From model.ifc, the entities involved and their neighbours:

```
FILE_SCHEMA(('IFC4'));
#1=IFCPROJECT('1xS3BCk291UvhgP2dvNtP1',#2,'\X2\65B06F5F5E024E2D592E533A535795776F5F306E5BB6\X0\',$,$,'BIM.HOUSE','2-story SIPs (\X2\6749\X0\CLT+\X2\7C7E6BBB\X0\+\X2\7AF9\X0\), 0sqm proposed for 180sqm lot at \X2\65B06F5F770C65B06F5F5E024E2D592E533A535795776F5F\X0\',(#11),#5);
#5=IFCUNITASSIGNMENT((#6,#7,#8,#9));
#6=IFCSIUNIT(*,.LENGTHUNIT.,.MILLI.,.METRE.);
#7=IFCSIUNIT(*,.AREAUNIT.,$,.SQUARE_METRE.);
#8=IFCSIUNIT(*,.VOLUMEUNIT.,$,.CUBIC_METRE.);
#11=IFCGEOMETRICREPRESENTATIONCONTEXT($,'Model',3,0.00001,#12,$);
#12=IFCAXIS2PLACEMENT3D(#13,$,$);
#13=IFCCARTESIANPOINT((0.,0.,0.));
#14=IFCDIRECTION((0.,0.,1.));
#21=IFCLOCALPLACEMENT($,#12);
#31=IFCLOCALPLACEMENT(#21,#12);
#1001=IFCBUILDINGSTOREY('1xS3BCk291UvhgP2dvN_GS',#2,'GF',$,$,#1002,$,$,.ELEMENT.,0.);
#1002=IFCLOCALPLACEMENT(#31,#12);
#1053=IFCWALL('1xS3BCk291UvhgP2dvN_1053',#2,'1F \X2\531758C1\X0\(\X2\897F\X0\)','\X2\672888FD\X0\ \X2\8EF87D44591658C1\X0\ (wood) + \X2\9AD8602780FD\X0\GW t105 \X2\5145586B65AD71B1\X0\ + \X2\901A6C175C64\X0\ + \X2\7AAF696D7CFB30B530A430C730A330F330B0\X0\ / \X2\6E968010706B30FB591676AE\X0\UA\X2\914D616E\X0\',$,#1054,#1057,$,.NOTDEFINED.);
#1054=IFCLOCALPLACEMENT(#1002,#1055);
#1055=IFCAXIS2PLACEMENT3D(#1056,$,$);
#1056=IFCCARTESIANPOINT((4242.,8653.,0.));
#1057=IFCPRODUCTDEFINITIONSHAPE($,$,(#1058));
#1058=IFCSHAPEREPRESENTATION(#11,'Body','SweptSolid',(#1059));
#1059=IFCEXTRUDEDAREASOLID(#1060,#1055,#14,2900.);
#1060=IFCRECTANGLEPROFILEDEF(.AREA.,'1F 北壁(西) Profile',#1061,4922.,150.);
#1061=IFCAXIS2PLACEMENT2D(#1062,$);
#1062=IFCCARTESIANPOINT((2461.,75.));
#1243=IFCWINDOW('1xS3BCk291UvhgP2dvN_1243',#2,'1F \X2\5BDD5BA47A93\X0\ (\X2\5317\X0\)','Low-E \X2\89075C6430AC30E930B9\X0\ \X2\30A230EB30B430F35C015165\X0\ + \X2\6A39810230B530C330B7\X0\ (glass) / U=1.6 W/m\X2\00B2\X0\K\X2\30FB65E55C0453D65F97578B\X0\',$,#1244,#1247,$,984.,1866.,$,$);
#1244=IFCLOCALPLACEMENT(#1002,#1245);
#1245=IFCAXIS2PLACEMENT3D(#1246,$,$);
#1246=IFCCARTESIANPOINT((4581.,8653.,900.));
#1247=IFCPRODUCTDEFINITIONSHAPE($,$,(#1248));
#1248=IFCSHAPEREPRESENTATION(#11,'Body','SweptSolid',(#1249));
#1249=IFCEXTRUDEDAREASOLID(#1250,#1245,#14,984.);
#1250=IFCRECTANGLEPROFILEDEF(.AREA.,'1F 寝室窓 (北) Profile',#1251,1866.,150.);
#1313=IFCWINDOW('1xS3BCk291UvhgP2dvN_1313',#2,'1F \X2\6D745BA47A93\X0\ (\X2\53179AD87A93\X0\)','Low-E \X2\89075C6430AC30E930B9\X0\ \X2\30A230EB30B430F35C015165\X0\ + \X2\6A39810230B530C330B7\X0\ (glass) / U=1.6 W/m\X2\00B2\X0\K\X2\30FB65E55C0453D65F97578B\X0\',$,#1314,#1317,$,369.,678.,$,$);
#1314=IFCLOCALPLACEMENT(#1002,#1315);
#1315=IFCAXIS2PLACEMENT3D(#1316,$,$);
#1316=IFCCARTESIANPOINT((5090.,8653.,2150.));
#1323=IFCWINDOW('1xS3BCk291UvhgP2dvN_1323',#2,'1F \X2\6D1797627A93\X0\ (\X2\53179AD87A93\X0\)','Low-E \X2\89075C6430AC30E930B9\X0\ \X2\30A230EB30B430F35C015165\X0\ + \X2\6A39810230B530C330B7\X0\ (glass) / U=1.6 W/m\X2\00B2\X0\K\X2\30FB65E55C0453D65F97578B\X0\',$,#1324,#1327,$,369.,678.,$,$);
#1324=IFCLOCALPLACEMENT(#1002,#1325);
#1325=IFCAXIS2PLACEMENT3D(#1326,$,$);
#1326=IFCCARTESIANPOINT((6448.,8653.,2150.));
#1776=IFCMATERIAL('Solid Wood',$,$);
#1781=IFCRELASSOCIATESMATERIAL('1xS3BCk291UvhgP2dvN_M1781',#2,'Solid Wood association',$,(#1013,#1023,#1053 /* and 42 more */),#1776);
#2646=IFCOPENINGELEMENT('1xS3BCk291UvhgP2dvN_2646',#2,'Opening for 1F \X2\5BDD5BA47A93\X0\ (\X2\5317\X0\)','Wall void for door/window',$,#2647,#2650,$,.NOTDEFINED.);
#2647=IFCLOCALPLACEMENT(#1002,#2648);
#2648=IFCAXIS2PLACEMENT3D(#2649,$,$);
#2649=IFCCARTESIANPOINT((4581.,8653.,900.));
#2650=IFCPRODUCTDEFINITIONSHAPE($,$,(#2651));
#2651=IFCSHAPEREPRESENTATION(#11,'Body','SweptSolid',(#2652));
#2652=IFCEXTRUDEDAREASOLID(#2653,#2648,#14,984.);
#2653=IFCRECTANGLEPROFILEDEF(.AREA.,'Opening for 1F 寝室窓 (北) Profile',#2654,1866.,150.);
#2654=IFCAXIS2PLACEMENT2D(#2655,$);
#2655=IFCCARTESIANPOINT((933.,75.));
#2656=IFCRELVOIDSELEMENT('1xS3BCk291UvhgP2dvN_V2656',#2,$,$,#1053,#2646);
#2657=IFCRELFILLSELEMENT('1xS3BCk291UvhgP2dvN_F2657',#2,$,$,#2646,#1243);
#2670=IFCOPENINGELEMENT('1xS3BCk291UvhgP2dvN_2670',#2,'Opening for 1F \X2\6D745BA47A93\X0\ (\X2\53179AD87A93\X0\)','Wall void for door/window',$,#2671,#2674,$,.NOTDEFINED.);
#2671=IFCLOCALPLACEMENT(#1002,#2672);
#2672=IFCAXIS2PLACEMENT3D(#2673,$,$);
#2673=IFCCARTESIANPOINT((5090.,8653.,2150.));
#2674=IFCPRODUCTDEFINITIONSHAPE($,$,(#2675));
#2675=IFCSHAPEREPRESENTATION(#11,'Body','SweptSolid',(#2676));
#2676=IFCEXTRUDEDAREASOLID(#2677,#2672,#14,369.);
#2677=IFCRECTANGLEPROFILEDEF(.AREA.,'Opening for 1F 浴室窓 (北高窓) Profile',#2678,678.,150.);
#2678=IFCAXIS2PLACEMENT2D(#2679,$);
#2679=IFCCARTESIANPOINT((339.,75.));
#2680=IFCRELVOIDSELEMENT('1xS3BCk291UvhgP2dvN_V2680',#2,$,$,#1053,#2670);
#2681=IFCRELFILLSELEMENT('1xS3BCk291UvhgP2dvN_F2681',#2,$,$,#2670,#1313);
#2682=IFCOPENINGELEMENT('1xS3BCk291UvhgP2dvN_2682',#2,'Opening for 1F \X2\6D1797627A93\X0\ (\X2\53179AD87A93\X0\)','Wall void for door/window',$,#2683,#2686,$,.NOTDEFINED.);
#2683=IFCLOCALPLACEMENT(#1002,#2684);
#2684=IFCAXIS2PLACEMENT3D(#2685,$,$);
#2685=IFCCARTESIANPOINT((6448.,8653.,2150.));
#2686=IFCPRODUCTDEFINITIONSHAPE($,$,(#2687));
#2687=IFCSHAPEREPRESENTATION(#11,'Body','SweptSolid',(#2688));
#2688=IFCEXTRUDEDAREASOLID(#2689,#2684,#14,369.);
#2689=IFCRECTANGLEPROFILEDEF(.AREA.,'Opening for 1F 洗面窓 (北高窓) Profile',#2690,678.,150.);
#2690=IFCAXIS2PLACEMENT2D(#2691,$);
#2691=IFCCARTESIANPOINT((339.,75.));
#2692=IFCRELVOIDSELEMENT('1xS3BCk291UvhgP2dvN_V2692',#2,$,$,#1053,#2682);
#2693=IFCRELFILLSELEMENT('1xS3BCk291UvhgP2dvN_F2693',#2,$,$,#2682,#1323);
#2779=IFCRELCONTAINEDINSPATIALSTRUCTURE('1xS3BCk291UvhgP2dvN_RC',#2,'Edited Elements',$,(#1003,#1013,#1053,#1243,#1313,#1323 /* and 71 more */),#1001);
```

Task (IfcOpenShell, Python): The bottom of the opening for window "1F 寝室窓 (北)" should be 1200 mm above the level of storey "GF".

```python
import numpy as np
import ifcopenshell
import ifcopenshell.api.geometry
import ifcopenshell.geom
import ifcopenshell.util.element
import ifcopenshell.util.placement
import ifcopenshell.util.shape
import ifcopenshell.util.unit

model = ifcopenshell.open("model.ifc")
unit_scale = ifcopenshell.util.unit.calculate_unit_scale(model)

window = model.by_guid("1xS3BCk291UvhgP2dvN_1243")
opening = window.FillsVoids[0].RelatingOpeningElement
storey = ifcopenshell.util.element.get_container(window, ifc_class="IfcBuildingStorey")
level = ifcopenshell.util.placement.get_local_placement(storey.ObjectPlacement)[2, 3]

# The opening's origin need not be at the sill, so measure its lowest point.
shape = ifcopenshell.geom.create_shape(ifcopenshell.geom.settings(), opening)
bottom = ifcopenshell.util.shape.get_shape_bottom_elevation(shape, shape.geometry) / unit_scale
dz = level + 1.2 / unit_scale - bottom

shift = np.array([0.0, 0.0, dz])
# The window is not placed relative to its opening, so move both.
for product in (opening, window):
    matrix = ifcopenshell.util.placement.get_local_placement(product.ObjectPlacement)
    matrix[:3, 3] += shift
    ifcopenshell.api.geometry.edit_object_placement(model, product=product, matrix=matrix, is_si=False)

print(f"moved by {dz * unit_scale:+.3f} m")

model.write("model_rev.ifc")
```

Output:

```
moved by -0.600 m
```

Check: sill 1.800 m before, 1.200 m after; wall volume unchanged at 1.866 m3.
